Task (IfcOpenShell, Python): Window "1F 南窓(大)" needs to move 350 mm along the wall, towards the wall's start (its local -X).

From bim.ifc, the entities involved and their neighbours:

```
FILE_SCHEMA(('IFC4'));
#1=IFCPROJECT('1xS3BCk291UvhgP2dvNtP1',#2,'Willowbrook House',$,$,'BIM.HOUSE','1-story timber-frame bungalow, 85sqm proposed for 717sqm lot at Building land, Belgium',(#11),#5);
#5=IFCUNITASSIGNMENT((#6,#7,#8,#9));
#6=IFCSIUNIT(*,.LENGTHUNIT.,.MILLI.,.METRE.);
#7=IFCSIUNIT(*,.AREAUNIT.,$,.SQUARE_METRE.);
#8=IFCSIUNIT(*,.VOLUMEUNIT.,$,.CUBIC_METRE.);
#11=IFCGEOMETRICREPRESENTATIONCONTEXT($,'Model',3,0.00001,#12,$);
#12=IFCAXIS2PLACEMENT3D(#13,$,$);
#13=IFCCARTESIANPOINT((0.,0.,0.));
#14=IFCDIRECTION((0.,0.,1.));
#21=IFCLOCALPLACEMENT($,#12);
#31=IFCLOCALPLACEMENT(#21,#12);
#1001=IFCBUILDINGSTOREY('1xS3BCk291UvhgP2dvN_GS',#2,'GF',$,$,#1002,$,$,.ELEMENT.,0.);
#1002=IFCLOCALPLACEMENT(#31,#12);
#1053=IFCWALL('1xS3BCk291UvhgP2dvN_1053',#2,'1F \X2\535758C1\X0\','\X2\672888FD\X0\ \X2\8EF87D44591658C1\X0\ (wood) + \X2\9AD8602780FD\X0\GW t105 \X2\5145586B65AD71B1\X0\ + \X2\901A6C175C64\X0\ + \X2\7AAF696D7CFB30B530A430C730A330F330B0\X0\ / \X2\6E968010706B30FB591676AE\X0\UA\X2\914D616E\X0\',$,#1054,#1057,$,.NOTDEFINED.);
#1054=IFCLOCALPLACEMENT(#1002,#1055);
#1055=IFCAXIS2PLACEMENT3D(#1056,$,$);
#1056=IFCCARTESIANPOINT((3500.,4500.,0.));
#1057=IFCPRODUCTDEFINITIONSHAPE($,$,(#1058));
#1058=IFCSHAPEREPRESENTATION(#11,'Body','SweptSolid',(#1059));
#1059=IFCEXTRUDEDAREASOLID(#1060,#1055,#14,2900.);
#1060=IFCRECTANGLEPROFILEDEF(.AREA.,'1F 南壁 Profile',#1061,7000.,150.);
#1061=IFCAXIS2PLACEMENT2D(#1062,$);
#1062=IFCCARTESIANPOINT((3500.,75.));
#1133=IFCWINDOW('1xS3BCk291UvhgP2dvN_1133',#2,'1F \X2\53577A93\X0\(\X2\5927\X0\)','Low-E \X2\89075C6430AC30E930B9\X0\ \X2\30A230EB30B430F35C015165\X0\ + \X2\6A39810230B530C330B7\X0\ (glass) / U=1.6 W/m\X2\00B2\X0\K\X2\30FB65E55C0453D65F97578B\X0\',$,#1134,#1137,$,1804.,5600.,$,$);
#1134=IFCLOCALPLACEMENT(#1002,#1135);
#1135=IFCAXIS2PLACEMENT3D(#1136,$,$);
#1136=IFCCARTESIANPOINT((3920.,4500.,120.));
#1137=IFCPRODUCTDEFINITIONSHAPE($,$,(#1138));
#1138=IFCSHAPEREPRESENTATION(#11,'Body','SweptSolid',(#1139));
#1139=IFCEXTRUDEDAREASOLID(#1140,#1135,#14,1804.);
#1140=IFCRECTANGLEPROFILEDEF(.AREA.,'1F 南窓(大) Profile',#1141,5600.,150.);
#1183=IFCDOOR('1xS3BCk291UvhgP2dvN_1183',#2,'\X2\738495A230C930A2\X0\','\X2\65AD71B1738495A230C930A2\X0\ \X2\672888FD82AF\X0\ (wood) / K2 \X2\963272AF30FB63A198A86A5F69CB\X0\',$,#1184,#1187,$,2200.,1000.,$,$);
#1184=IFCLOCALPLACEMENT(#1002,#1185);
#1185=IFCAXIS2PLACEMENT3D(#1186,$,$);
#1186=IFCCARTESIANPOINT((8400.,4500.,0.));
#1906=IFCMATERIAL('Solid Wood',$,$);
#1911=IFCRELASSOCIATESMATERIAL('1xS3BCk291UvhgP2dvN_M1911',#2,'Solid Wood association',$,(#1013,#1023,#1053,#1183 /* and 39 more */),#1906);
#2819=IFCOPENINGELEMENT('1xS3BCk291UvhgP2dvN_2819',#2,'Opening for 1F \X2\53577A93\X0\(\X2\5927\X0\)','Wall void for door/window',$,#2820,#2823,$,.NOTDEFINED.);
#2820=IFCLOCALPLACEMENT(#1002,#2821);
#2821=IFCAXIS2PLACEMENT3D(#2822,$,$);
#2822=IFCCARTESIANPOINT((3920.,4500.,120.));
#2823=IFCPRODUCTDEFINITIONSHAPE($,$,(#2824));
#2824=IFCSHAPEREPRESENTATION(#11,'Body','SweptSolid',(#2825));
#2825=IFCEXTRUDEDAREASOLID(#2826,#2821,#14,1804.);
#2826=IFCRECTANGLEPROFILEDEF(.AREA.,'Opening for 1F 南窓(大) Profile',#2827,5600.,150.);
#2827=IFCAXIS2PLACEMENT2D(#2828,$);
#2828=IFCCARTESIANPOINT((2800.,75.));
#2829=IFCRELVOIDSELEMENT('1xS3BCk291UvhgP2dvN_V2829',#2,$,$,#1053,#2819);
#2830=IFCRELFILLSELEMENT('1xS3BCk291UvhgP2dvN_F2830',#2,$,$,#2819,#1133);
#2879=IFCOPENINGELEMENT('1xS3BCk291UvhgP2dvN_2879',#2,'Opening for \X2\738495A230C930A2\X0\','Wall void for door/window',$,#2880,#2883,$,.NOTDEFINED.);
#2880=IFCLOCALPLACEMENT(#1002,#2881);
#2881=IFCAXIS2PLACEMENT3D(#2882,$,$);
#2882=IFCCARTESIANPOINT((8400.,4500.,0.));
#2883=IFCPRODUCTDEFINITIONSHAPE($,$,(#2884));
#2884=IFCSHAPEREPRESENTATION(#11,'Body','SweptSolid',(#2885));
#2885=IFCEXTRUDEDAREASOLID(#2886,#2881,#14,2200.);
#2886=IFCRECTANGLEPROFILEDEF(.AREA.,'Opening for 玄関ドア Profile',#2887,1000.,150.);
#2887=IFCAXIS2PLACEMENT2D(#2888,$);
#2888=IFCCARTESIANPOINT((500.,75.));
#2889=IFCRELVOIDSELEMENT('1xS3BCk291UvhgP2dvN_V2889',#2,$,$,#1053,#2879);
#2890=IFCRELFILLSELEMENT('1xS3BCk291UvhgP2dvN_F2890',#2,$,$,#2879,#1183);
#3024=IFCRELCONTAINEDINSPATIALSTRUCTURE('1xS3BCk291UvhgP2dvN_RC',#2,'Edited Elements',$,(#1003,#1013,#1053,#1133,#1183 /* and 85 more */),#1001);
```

```python
import ifcopenshell
import ifcopenshell.api.geometry
import ifcopenshell.util.placement
import ifcopenshell.util.unit

model = ifcopenshell.open("bim.ifc")
unit_scale = ifcopenshell.util.unit.calculate_unit_scale(model)

window = model.by_guid("1xS3BCk291UvhgP2dvN_1133")
opening = window.FillsVoids[0].RelatingOpeningElement
wall = opening.VoidsElements[0].RelatingBuildingElement

wall_matrix = ifcopenshell.util.placement.get_local_placement(wall.ObjectPlacement)
shift = wall_matrix[:3, 0] * -0.35 / unit_scale
before = ifcopenshell.util.placement.get_local_placement(window.ObjectPlacement)[:3, 3].copy()

# The window is not placed relative to its opening, so move both.
for product in (opening, window):
    matrix = ifcopenshell.util.placement.get_local_placement(product.ObjectPlacement)
    matrix[:3, 3] += shift
    ifcopenshell.api.geometry.edit_object_placement(model, product=product, matrix=matrix, is_si=False)

after = ifcopenshell.util.placement.get_local_placement(window.ObjectPlacement)[:3, 3]
print("window moved by", (after - before).round(3) + 0.0)

model.write("bim_updated.ifc")
```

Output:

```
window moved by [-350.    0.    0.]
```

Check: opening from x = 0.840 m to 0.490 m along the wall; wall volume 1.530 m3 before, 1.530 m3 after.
